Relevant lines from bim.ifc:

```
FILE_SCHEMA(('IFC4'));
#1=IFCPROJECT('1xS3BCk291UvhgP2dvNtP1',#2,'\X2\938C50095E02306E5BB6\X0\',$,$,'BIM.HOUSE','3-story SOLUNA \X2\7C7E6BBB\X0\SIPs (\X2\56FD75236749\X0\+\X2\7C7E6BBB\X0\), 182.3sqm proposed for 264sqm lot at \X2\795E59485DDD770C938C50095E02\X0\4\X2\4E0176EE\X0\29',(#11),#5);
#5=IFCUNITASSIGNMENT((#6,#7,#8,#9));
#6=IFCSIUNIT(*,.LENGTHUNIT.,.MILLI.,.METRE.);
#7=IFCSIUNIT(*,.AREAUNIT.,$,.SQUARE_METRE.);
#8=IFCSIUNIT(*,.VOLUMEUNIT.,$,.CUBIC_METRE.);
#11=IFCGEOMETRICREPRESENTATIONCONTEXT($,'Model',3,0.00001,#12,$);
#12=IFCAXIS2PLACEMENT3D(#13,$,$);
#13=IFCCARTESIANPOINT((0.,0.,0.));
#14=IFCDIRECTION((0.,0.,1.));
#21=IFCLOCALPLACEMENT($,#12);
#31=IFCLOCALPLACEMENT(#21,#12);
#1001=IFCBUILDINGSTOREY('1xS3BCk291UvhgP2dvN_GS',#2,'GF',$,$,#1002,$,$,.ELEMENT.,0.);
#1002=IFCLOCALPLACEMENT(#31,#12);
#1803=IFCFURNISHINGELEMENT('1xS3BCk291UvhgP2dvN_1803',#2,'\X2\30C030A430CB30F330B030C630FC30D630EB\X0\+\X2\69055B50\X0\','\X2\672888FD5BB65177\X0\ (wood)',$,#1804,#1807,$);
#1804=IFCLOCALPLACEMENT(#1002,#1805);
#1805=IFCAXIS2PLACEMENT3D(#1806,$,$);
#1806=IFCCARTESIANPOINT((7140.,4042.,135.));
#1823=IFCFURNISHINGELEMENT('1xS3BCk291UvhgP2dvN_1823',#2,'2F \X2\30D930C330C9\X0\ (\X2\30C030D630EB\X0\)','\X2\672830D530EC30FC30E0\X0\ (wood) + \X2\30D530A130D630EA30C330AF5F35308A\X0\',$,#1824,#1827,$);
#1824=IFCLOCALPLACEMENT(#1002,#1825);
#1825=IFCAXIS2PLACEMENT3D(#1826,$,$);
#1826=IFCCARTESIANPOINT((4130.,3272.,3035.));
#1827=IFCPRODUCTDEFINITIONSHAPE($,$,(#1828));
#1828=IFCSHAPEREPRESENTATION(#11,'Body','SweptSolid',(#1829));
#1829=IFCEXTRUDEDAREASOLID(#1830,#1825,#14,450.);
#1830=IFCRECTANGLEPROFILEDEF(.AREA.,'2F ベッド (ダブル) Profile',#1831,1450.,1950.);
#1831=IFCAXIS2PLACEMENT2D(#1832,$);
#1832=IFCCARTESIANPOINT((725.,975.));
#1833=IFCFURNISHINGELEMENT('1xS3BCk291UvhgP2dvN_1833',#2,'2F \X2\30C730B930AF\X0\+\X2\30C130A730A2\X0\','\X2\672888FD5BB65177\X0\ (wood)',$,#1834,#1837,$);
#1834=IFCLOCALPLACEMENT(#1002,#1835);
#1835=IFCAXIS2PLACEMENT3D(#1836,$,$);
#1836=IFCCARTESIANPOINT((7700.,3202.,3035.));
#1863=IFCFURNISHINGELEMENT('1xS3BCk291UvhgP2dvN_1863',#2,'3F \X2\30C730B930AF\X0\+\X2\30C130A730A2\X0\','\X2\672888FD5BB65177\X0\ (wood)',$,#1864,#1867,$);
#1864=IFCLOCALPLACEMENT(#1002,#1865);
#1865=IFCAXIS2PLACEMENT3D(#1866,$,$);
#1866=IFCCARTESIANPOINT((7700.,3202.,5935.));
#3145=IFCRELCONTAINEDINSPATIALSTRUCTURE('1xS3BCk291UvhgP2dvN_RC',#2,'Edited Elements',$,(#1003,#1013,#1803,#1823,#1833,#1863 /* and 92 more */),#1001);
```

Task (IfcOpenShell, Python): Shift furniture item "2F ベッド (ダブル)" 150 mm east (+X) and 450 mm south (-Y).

```python
import ifcopenshell
import ifcopenshell.api.geometry
import ifcopenshell.util.placement
import ifcopenshell.util.unit

model = ifcopenshell.open("bim.ifc")
unit_scale = ifcopenshell.util.unit.calculate_unit_scale(model)

item = model.by_guid("1xS3BCk291UvhgP2dvN_1823")
matrix = ifcopenshell.util.placement.get_local_placement(item.ObjectPlacement)
matrix[0, 3] += 0.15 / unit_scale
matrix[1, 3] -= 0.45 / unit_scale
ifcopenshell.api.geometry.edit_object_placement(model, product=item, matrix=matrix, is_si=False)

print(ifcopenshell.util.placement.get_local_placement(item.ObjectPlacement).round(3) + 0.0)

model.write("bim_updated.ifc")
```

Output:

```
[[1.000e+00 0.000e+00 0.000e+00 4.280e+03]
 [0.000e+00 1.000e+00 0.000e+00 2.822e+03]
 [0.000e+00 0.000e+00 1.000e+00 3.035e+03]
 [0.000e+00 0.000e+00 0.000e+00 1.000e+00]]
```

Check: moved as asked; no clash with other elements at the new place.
